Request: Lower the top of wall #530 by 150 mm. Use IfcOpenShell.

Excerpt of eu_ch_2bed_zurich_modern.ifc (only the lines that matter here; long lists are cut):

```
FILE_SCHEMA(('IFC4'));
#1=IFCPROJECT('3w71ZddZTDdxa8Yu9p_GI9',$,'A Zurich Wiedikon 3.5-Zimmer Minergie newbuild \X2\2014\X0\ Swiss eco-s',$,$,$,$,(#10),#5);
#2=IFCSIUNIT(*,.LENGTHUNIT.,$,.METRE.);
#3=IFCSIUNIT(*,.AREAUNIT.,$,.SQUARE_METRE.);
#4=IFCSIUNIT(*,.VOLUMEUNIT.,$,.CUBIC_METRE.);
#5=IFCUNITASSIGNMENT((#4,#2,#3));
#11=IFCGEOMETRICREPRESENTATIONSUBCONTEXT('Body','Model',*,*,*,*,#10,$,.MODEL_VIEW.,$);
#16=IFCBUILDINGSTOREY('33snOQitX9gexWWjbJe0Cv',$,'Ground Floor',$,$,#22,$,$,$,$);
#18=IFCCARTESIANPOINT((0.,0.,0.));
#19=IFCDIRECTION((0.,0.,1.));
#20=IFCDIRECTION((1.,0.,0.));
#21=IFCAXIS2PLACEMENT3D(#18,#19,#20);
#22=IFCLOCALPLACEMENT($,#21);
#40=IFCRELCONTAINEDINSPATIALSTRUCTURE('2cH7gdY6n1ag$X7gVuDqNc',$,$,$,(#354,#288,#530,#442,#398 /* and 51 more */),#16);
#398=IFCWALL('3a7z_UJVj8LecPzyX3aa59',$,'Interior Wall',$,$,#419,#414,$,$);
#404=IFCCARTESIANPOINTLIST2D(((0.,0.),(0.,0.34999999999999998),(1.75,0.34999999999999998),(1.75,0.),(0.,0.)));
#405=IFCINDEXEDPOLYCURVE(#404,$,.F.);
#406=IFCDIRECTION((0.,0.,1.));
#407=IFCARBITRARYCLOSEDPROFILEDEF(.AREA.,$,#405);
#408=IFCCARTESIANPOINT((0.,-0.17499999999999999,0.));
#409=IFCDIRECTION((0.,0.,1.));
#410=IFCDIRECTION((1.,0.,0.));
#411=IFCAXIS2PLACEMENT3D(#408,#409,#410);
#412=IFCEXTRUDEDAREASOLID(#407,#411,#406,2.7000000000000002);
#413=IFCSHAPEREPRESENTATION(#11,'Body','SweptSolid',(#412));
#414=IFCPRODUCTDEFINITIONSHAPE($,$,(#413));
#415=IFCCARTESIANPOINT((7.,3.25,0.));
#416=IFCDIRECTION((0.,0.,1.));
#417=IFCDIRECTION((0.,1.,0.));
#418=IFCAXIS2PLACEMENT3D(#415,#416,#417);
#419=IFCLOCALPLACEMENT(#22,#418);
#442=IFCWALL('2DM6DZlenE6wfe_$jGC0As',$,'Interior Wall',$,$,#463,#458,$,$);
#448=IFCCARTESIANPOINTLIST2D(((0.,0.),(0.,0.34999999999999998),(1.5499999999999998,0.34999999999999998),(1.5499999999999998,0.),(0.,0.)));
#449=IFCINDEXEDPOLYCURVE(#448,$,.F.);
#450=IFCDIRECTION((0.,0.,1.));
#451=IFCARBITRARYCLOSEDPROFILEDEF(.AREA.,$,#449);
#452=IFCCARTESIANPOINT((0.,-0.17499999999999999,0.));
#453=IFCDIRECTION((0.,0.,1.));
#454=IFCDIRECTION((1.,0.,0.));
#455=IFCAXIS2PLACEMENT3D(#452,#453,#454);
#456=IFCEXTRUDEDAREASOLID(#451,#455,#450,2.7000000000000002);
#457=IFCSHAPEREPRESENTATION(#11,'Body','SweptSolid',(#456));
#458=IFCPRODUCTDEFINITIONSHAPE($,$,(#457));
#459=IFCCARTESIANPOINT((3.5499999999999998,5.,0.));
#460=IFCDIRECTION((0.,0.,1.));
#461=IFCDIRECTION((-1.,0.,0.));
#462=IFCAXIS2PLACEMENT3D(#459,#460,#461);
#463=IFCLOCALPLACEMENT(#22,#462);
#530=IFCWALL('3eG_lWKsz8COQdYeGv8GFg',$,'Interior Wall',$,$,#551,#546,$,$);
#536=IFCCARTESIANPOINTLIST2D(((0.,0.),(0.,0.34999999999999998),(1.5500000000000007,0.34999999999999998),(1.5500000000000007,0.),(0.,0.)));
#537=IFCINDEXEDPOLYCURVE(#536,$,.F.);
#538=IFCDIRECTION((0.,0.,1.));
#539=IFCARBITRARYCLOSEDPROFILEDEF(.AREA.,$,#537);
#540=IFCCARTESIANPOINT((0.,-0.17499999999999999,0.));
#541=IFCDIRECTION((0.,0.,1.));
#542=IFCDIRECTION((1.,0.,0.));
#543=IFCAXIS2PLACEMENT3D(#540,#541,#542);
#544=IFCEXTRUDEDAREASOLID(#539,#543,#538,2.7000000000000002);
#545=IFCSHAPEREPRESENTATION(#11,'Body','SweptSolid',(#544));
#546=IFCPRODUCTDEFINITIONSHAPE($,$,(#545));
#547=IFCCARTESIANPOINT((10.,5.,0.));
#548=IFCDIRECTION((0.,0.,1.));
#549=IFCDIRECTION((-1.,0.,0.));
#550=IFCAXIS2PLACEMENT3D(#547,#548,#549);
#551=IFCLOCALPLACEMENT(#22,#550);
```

```python
import ifcopenshell
import ifcopenshell.geom
import ifcopenshell.util.representation
import ifcopenshell.util.shape
import ifcopenshell.util.unit

model = ifcopenshell.open("eu_ch_2bed_zurich_modern.ifc")
unit_scale = ifcopenshell.util.unit.calculate_unit_scale(model)
settings = ifcopenshell.geom.settings()


def volume(element):
    """Net volume in cubic metres, openings subtracted."""
    shape = ifcopenshell.geom.create_shape(settings, element)
    return ifcopenshell.util.shape.get_volume(shape.geometry)


wall = model.by_guid("3eG_lWKsz8COQdYeGv8GFg")
before = volume(wall)

body = ifcopenshell.util.representation.get_representation(wall, "Model", "Body")
solid = body.Items[0]
old_height = solid.Depth
solid.Depth -= 0.15 / unit_scale
after = volume(wall)

print(f"height {old_height:g} -> {solid.Depth:g}, volume {before:.3f} -> {after:.3f} m3")

model.write("eu_ch_2bed_zurich_modern_updated.ifc")
```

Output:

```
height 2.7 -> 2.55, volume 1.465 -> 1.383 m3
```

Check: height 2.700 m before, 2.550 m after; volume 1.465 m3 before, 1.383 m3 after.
